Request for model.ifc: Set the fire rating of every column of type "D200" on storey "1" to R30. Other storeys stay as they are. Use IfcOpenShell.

First a look at what the model holds.

```python
import ifcopenshell
import ifcopenshell.util.element

model = ifcopenshell.open("model.ifc")
print(model.schema)
storey = next(s for s in model.by_type("IfcBuildingStorey") if s.Name == "1")
columns = [e for e in ifcopenshell.util.element.get_decomposition(storey) if e.is_a("IfcColumn")]
seen = {}
for e in columns:
    element_type = ifcopenshell.util.element.get_type(e)
    key = (element_type.Name if element_type != e and element_type else None, ifcopenshell.util.element.get_pset(e, "Pset_ColumnCommon", "FireRating"))
    seen[key] = seen.get(key, 0) + 1
for (name, value), count in sorted(seen.items(), key=str):
    print(count, "x", name, "|", value)
```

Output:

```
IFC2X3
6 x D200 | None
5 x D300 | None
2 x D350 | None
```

```python
import ifcopenshell
import ifcopenshell.api.pset
import ifcopenshell.util.element

model = ifcopenshell.open("model.ifc")

storey = next(s for s in model.by_type("IfcBuildingStorey") if s.Name == "1")
columns = [e for e in ifcopenshell.util.element.get_decomposition(storey) if e.is_a("IfcColumn")]

count = 0
for e in columns:
    element_type = ifcopenshell.util.element.get_type(e)
    if element_type in (None, e) or element_type.Name != "D200":
        continue
    # add_pset returns the element's existing set when there is one.
    pset = ifcopenshell.api.pset.add_pset(model, product=e, name="Pset_ColumnCommon")
    ifcopenshell.api.pset.edit_pset(model, pset=pset, properties={"FireRating": "R30"})
    count += 1

print(count, "columns updated")

model.write("model-out.ifc")
```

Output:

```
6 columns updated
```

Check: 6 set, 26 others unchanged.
